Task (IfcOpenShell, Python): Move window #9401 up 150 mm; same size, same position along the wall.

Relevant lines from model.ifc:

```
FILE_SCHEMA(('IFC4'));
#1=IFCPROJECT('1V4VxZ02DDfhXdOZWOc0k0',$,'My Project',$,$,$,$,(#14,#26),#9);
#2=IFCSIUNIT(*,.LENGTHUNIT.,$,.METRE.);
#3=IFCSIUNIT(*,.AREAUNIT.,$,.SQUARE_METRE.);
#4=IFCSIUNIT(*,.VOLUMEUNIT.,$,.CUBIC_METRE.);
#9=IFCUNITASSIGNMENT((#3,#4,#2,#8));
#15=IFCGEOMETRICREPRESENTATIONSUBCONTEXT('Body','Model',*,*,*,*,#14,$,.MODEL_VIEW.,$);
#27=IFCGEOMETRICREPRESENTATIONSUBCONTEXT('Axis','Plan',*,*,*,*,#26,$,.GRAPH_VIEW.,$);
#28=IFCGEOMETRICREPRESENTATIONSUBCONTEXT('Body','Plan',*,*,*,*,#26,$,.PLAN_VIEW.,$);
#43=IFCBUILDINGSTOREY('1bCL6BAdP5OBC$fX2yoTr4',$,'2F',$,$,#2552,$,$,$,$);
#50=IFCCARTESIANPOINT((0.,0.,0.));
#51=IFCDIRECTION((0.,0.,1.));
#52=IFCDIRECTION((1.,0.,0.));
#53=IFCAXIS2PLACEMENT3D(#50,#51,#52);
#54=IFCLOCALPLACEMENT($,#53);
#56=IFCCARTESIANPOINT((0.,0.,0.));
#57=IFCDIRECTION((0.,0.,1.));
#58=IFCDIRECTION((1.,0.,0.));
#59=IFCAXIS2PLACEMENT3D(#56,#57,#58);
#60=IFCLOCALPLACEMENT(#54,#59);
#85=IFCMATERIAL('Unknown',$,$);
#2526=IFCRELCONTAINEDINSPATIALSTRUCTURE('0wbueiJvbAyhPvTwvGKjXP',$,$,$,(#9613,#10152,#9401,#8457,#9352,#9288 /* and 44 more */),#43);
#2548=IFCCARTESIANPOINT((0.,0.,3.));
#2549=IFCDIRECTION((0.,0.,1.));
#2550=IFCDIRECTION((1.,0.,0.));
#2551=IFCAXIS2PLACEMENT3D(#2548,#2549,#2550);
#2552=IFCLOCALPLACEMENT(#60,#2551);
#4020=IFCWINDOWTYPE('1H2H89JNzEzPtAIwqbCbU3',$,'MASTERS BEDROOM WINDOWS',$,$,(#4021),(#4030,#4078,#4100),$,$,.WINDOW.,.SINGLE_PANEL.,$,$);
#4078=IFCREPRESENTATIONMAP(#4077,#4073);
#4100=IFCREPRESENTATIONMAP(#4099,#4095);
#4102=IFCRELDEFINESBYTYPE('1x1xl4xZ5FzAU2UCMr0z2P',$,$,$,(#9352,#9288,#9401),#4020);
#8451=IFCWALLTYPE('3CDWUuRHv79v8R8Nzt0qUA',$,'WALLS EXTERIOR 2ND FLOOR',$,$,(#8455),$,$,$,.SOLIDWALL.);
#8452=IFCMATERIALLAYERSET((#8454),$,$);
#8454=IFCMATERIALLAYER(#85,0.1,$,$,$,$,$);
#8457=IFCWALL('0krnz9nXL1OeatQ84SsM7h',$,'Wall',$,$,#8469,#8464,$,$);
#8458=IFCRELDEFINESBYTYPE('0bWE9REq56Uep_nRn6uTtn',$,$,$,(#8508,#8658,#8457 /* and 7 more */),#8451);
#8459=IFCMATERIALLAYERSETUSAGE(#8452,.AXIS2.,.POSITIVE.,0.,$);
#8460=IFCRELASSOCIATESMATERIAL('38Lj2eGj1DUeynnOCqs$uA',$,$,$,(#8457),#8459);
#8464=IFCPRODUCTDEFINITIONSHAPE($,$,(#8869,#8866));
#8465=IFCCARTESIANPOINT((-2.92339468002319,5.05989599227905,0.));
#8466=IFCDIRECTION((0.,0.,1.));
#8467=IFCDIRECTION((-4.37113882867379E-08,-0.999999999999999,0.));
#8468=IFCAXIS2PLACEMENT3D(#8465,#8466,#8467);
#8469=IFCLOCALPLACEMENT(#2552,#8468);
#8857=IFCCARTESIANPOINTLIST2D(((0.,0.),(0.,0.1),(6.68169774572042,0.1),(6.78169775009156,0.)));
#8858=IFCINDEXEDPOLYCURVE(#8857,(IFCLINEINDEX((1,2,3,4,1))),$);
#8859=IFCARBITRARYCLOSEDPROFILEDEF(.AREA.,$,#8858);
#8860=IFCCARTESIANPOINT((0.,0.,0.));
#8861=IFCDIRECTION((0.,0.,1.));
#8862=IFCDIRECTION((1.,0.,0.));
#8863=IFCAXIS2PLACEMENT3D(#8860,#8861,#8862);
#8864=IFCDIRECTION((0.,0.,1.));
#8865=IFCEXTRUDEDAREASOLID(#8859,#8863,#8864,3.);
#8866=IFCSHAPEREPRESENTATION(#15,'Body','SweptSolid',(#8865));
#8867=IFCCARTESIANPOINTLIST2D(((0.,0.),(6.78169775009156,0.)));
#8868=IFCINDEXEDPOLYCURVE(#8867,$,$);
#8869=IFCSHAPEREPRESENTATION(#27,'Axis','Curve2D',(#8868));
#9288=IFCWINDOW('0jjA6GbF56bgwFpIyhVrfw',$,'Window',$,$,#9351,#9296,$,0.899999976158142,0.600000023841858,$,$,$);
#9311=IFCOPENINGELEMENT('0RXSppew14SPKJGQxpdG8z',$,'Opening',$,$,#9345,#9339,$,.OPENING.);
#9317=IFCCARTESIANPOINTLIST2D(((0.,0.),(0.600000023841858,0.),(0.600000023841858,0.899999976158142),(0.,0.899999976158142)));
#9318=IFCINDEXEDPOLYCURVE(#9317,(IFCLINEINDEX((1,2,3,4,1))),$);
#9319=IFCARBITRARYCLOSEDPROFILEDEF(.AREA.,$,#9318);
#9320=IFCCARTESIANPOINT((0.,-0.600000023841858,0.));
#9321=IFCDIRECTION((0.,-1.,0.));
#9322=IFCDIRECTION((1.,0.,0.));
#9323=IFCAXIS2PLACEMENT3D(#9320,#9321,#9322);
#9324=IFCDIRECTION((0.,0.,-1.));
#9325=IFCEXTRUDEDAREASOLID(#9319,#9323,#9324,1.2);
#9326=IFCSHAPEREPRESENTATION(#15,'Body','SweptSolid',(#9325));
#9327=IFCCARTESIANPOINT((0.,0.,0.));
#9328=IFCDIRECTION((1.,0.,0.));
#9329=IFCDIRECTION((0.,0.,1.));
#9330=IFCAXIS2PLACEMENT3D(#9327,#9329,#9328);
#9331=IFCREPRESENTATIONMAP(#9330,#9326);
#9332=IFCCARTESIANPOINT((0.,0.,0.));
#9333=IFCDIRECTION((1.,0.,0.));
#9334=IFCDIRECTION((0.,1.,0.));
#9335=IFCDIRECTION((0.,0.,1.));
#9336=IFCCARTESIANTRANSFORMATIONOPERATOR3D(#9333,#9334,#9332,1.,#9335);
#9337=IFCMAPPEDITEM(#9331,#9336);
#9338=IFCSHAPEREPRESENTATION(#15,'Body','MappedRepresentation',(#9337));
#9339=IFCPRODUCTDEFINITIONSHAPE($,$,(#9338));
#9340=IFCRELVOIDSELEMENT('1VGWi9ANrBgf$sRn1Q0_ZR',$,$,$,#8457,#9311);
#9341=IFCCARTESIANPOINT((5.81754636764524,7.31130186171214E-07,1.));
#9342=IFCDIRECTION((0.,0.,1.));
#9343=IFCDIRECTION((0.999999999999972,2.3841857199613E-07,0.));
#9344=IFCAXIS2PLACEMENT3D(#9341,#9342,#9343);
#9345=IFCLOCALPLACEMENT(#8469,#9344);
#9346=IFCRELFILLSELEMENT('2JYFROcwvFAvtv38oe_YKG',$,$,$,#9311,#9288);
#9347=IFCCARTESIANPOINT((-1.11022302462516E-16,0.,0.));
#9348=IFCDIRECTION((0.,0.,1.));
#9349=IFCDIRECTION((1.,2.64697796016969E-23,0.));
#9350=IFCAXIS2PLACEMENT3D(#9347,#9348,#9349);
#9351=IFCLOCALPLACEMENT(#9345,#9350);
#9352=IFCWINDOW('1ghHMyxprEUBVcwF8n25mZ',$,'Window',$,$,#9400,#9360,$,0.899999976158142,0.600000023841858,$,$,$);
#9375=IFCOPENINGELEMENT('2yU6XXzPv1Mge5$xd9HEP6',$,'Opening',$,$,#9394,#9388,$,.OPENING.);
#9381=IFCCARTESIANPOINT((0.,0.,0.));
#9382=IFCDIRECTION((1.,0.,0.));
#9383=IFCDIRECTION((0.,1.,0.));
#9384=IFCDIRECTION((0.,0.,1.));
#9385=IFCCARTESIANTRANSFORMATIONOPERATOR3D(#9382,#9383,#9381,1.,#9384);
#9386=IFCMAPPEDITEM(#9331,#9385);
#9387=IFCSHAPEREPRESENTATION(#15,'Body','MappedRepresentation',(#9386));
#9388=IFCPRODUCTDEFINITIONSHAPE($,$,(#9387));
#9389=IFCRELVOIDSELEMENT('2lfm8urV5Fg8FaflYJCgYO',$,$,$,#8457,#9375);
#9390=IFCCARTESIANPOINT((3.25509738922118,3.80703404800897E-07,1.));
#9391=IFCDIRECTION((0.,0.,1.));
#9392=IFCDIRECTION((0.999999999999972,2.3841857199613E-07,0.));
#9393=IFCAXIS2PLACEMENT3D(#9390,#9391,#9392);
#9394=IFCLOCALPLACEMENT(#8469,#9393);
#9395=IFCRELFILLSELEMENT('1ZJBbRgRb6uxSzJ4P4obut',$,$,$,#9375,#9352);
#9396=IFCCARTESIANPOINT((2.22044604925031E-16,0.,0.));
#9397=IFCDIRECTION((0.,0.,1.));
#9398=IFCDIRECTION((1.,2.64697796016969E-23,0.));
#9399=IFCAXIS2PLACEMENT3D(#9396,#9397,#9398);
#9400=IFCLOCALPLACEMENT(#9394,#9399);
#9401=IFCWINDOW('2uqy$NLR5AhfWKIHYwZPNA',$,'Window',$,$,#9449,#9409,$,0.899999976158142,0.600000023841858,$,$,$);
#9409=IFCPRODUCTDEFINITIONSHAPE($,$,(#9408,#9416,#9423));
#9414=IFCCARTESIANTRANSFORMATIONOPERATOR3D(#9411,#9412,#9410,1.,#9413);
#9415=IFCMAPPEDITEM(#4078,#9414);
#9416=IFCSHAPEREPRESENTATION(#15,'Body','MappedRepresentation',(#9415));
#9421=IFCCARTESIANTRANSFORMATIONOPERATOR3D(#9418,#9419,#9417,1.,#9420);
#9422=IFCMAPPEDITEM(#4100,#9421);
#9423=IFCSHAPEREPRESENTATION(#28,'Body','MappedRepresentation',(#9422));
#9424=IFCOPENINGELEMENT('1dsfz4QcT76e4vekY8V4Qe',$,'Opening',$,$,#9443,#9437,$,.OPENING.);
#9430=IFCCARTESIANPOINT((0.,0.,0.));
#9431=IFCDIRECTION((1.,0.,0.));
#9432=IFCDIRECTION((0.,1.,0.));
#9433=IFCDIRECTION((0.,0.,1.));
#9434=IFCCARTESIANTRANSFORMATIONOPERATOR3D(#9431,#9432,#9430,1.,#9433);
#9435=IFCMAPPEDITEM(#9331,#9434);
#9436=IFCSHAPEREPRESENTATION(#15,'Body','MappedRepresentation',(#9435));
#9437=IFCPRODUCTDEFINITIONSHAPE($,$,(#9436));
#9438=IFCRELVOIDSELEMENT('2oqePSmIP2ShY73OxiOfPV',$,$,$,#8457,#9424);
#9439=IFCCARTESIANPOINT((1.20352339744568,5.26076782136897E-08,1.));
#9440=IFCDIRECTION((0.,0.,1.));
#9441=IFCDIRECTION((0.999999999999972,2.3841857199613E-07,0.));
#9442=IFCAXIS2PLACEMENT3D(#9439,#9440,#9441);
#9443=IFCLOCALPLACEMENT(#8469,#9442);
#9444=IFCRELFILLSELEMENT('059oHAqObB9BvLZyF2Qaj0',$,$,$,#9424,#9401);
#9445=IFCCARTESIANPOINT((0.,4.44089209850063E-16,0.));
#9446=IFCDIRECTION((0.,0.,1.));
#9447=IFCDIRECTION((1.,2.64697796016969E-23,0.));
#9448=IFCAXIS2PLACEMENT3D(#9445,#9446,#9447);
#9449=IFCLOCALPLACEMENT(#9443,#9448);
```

```python
import numpy as np
import ifcopenshell
import ifcopenshell.api.geometry
import ifcopenshell.util.placement
import ifcopenshell.util.unit

model = ifcopenshell.open("model.ifc")
unit_scale = ifcopenshell.util.unit.calculate_unit_scale(model)

window = model.by_guid("2uqy$NLR5AhfWKIHYwZPNA")
opening = window.FillsVoids[0].RelatingOpeningElement
dz = 0.15

shift = np.array([0.0, 0.0, dz])
# The window is placed relative to its opening, so it follows when the opening moves.
matrix = ifcopenshell.util.placement.get_local_placement(opening.ObjectPlacement)
matrix[:3, 3] += shift
ifcopenshell.api.geometry.edit_object_placement(
    model, product=opening, matrix=matrix, is_si=False, should_transform_children=True
)

print(f"moved by {dz * unit_scale:+.3f} m")

model.write("model_v2.ifc")
```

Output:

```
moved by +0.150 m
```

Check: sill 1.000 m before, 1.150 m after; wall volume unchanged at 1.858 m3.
